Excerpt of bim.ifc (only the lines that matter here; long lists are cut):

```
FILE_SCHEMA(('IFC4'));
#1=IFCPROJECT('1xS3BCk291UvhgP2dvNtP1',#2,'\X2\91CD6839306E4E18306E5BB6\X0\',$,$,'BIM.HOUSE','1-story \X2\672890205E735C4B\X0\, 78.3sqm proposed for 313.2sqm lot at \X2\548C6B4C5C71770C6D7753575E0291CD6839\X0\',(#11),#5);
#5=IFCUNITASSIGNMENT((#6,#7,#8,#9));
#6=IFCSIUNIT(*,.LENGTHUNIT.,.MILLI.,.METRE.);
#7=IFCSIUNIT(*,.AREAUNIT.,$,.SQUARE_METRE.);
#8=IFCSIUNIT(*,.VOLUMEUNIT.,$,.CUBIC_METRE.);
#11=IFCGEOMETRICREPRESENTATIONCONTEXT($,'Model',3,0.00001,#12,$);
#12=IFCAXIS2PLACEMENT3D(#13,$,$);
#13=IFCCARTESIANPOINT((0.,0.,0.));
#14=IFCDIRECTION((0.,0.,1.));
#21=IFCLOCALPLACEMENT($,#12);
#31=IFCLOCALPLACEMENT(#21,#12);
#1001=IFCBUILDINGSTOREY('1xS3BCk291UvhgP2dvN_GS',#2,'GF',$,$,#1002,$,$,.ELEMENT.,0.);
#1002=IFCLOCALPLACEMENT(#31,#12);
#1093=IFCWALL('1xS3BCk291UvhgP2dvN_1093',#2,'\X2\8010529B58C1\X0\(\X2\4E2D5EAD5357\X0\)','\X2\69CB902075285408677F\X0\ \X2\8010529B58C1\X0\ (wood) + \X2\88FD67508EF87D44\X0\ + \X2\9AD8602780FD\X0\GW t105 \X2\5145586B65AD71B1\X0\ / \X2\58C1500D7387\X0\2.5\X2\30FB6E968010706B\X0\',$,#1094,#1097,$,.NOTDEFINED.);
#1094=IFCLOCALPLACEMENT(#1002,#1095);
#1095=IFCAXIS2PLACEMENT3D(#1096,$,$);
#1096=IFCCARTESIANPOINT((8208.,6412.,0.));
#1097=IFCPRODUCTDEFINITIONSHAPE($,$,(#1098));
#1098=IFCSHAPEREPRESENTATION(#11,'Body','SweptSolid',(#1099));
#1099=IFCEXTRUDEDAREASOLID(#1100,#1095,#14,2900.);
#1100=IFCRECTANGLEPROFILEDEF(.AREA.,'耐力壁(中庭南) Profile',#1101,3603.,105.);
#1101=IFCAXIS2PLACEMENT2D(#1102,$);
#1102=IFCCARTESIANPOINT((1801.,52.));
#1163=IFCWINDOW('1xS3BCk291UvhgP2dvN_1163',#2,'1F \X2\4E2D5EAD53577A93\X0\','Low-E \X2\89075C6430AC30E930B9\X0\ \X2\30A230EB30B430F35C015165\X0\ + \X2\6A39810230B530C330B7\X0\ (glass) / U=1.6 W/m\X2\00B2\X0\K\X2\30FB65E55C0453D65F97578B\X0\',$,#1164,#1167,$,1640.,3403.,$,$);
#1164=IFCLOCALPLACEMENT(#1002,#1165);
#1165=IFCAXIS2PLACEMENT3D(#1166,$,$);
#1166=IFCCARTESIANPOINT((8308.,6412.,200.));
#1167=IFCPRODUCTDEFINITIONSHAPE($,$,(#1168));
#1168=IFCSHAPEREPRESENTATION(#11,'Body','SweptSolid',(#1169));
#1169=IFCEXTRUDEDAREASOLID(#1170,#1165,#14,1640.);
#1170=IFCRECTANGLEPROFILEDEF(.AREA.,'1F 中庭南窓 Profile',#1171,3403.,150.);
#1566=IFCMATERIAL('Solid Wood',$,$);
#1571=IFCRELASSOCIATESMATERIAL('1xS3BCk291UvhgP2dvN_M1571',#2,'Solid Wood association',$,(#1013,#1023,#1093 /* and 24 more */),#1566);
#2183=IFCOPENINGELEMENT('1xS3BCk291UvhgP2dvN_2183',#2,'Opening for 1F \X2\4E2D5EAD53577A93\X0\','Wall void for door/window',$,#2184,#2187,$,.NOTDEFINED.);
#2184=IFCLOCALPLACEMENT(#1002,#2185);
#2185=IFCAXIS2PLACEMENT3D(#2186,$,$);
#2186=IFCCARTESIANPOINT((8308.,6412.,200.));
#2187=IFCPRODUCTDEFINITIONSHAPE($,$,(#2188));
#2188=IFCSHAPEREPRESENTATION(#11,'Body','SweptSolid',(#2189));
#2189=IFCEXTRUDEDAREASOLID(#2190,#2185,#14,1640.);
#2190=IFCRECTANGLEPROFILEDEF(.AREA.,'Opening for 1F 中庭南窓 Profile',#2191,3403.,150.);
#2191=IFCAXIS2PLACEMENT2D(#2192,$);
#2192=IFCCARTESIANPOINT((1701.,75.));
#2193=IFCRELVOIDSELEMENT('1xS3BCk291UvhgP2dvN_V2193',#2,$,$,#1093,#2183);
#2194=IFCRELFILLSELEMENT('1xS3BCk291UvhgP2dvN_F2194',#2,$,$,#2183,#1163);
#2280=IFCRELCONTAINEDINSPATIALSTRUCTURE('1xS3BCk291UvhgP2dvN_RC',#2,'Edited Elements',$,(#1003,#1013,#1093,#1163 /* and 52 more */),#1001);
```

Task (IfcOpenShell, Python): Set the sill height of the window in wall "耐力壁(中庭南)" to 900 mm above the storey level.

```python
import numpy as np
import ifcopenshell
import ifcopenshell.api.geometry
import ifcopenshell.geom
import ifcopenshell.util.element
import ifcopenshell.util.placement
import ifcopenshell.util.shape
import ifcopenshell.util.unit

model = ifcopenshell.open("bim.ifc")
unit_scale = ifcopenshell.util.unit.calculate_unit_scale(model)

window = model.by_guid("1xS3BCk291UvhgP2dvN_1163")
opening = window.FillsVoids[0].RelatingOpeningElement
storey = ifcopenshell.util.element.get_container(window, ifc_class="IfcBuildingStorey")
level = ifcopenshell.util.placement.get_local_placement(storey.ObjectPlacement)[2, 3]

# The opening's origin need not be at the sill, so measure its lowest point.
shape = ifcopenshell.geom.create_shape(ifcopenshell.geom.settings(), opening)
bottom = ifcopenshell.util.shape.get_shape_bottom_elevation(shape, shape.geometry) / unit_scale
dz = level + 900.0 - bottom

shift = np.array([0.0, 0.0, dz])
# The window is not placed relative to its opening, so move both.
for product in (opening, window):
    matrix = ifcopenshell.util.placement.get_local_placement(product.ObjectPlacement)
    matrix[:3, 3] += shift
    ifcopenshell.api.geometry.edit_object_placement(model, product=product, matrix=matrix, is_si=False)

print(f"moved by {dz * unit_scale:+.3f} m")

model.write("bim_v2.ifc")
```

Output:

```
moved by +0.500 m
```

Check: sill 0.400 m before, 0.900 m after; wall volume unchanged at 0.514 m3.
